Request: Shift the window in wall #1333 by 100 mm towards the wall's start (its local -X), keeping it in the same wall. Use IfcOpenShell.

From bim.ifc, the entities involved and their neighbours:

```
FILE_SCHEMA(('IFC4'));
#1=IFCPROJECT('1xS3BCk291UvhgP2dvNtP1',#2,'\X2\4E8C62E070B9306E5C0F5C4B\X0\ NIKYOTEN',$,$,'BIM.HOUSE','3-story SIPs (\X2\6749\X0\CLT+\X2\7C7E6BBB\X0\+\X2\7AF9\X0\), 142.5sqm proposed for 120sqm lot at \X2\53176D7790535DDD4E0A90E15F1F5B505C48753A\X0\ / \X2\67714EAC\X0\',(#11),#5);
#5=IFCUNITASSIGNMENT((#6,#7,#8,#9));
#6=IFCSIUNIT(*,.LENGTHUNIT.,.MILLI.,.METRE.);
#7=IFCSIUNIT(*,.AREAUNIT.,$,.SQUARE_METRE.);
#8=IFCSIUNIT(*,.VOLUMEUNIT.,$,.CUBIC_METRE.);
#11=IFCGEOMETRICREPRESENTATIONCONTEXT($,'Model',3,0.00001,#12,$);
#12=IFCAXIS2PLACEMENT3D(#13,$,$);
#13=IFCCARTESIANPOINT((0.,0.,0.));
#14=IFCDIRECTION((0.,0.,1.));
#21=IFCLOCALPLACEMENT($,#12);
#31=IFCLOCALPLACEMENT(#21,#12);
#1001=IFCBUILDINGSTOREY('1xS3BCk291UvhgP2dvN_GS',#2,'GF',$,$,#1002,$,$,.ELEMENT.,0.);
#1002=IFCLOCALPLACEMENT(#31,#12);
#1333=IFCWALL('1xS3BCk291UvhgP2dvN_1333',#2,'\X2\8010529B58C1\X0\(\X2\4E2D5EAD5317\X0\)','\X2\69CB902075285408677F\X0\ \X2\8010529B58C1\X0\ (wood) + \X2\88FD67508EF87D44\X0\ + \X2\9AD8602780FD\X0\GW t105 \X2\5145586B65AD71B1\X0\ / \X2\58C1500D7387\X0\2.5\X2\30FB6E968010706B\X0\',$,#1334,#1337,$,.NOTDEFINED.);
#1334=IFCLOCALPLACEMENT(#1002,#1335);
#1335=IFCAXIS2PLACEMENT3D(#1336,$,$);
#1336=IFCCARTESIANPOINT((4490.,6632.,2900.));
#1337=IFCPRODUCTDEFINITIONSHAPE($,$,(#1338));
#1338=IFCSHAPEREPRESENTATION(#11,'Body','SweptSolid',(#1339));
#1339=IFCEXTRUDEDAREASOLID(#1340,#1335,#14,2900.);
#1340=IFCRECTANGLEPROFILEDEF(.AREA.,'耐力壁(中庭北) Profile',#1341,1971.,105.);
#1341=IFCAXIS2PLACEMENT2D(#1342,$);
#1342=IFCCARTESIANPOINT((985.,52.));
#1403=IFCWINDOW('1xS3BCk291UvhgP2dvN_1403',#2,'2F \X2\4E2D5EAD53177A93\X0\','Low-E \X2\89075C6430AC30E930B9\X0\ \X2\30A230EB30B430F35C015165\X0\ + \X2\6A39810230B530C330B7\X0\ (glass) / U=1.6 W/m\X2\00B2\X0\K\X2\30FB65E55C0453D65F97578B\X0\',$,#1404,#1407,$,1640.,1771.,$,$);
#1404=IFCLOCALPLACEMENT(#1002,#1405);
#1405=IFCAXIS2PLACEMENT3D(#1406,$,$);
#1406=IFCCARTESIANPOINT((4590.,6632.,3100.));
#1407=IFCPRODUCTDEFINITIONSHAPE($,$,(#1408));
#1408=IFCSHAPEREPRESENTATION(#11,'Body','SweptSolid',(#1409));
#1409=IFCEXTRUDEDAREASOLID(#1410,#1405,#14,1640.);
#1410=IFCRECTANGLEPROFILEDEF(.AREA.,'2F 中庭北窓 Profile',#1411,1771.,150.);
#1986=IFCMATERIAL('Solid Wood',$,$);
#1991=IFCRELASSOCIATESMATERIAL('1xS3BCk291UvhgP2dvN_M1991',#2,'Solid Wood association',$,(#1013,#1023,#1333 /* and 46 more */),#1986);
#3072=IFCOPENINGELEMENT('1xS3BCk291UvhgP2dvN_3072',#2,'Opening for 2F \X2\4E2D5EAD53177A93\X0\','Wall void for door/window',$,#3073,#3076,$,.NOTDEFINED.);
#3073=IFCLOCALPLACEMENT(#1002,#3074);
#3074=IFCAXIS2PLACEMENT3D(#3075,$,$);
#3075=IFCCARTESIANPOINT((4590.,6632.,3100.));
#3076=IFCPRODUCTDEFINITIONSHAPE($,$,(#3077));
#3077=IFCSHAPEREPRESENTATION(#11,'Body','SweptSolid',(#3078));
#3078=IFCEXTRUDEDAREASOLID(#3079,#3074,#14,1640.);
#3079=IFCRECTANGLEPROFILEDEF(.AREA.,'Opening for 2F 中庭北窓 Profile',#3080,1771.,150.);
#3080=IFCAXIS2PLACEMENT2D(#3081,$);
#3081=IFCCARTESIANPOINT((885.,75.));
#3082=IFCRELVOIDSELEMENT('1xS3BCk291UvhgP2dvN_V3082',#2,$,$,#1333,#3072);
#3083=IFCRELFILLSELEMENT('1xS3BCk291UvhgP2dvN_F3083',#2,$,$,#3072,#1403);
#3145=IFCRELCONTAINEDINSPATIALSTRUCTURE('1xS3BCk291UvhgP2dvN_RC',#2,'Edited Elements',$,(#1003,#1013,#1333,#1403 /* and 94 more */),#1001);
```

```python
import ifcopenshell
import ifcopenshell.api.geometry
import ifcopenshell.util.placement
import ifcopenshell.util.unit

model = ifcopenshell.open("bim.ifc")
unit_scale = ifcopenshell.util.unit.calculate_unit_scale(model)

window = model.by_guid("1xS3BCk291UvhgP2dvN_1403")
opening = window.FillsVoids[0].RelatingOpeningElement
wall = opening.VoidsElements[0].RelatingBuildingElement

wall_matrix = ifcopenshell.util.placement.get_local_placement(wall.ObjectPlacement)
shift = wall_matrix[:3, 0] * -0.1 / unit_scale
before = ifcopenshell.util.placement.get_local_placement(window.ObjectPlacement)[:3, 3].copy()

# The window is not placed relative to its opening, so move both.
for product in (opening, window):
    matrix = ifcopenshell.util.placement.get_local_placement(product.ObjectPlacement)
    matrix[:3, 3] += shift
    ifcopenshell.api.geometry.edit_object_placement(model, product=product, matrix=matrix, is_si=False)

after = ifcopenshell.util.placement.get_local_placement(window.ObjectPlacement)[:3, 3]
print("window moved by", (after - before).round(3) + 0.0)

model.write("bim_updated.ifc")
```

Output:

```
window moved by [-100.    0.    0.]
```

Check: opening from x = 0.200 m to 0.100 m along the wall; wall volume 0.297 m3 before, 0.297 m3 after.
